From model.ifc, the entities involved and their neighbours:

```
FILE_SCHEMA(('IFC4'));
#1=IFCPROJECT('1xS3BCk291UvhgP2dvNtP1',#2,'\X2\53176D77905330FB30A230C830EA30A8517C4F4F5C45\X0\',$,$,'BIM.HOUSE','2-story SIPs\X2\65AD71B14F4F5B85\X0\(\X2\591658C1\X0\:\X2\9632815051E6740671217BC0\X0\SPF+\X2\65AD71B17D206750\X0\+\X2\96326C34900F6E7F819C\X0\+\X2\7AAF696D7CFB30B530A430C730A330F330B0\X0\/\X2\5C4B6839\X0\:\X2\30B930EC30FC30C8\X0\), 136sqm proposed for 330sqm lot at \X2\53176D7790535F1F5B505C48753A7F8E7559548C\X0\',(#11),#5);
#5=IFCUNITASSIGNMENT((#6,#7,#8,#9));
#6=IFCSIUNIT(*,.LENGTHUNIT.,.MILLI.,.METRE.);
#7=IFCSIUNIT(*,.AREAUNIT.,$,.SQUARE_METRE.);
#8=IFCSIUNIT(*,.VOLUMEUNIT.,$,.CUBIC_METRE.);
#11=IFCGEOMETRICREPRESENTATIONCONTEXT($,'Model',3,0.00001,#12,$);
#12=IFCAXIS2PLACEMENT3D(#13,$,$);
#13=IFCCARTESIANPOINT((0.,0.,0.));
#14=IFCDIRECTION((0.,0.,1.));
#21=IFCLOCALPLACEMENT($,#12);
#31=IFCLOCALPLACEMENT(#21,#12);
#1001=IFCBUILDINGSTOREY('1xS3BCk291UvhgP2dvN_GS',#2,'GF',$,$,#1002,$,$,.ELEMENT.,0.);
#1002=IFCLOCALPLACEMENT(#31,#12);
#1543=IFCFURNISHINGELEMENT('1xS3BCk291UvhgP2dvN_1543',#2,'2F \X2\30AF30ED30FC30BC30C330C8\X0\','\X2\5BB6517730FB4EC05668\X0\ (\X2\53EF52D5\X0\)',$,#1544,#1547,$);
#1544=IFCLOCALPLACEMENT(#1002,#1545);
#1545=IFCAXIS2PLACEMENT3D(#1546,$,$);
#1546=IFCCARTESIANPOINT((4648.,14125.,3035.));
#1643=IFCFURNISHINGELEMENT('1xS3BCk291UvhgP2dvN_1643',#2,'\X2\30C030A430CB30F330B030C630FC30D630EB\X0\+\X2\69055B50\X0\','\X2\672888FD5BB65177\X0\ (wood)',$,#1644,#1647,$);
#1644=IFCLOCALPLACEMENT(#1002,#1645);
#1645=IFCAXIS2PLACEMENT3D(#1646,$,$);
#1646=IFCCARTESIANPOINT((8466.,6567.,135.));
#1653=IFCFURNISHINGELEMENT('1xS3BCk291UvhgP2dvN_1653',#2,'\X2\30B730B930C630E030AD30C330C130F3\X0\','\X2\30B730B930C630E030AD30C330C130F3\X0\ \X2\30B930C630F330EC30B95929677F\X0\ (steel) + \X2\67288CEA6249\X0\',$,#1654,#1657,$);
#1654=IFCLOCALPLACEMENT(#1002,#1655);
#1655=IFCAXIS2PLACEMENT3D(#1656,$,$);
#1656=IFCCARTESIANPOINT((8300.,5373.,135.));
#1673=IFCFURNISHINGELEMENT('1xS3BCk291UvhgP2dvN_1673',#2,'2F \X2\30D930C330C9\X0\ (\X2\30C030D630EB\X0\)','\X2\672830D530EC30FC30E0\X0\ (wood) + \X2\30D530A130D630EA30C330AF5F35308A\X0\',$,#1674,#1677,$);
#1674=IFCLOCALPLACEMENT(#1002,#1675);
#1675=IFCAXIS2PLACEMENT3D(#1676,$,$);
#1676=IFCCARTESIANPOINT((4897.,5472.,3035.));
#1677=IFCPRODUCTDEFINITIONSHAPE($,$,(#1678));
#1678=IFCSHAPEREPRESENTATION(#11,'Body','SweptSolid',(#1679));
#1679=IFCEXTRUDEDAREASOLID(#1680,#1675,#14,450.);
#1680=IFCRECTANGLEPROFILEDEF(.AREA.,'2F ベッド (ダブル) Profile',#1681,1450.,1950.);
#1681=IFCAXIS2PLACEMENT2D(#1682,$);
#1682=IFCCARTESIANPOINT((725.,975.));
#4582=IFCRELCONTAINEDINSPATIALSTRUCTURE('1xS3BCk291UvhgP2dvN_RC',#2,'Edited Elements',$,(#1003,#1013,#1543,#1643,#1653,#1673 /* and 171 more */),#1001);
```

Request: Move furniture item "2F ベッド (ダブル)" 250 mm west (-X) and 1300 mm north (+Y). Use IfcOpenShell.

```python
import ifcopenshell
import ifcopenshell.api.geometry
import ifcopenshell.util.placement
import ifcopenshell.util.unit

model = ifcopenshell.open("model.ifc")
unit_scale = ifcopenshell.util.unit.calculate_unit_scale(model)

item = model.by_id(1673)
matrix = ifcopenshell.util.placement.get_local_placement(item.ObjectPlacement)
matrix[0, 3] -= 0.25 / unit_scale
matrix[1, 3] += 1.3 / unit_scale
ifcopenshell.api.geometry.edit_object_placement(model, product=item, matrix=matrix, is_si=False)

print(ifcopenshell.util.placement.get_local_placement(item.ObjectPlacement).round(3) + 0.0)

model.write("model_edited.ifc")
```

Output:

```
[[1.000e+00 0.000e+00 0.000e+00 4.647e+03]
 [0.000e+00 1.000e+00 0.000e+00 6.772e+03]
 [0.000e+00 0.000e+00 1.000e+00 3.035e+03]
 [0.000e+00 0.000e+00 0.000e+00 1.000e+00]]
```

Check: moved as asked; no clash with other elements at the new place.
